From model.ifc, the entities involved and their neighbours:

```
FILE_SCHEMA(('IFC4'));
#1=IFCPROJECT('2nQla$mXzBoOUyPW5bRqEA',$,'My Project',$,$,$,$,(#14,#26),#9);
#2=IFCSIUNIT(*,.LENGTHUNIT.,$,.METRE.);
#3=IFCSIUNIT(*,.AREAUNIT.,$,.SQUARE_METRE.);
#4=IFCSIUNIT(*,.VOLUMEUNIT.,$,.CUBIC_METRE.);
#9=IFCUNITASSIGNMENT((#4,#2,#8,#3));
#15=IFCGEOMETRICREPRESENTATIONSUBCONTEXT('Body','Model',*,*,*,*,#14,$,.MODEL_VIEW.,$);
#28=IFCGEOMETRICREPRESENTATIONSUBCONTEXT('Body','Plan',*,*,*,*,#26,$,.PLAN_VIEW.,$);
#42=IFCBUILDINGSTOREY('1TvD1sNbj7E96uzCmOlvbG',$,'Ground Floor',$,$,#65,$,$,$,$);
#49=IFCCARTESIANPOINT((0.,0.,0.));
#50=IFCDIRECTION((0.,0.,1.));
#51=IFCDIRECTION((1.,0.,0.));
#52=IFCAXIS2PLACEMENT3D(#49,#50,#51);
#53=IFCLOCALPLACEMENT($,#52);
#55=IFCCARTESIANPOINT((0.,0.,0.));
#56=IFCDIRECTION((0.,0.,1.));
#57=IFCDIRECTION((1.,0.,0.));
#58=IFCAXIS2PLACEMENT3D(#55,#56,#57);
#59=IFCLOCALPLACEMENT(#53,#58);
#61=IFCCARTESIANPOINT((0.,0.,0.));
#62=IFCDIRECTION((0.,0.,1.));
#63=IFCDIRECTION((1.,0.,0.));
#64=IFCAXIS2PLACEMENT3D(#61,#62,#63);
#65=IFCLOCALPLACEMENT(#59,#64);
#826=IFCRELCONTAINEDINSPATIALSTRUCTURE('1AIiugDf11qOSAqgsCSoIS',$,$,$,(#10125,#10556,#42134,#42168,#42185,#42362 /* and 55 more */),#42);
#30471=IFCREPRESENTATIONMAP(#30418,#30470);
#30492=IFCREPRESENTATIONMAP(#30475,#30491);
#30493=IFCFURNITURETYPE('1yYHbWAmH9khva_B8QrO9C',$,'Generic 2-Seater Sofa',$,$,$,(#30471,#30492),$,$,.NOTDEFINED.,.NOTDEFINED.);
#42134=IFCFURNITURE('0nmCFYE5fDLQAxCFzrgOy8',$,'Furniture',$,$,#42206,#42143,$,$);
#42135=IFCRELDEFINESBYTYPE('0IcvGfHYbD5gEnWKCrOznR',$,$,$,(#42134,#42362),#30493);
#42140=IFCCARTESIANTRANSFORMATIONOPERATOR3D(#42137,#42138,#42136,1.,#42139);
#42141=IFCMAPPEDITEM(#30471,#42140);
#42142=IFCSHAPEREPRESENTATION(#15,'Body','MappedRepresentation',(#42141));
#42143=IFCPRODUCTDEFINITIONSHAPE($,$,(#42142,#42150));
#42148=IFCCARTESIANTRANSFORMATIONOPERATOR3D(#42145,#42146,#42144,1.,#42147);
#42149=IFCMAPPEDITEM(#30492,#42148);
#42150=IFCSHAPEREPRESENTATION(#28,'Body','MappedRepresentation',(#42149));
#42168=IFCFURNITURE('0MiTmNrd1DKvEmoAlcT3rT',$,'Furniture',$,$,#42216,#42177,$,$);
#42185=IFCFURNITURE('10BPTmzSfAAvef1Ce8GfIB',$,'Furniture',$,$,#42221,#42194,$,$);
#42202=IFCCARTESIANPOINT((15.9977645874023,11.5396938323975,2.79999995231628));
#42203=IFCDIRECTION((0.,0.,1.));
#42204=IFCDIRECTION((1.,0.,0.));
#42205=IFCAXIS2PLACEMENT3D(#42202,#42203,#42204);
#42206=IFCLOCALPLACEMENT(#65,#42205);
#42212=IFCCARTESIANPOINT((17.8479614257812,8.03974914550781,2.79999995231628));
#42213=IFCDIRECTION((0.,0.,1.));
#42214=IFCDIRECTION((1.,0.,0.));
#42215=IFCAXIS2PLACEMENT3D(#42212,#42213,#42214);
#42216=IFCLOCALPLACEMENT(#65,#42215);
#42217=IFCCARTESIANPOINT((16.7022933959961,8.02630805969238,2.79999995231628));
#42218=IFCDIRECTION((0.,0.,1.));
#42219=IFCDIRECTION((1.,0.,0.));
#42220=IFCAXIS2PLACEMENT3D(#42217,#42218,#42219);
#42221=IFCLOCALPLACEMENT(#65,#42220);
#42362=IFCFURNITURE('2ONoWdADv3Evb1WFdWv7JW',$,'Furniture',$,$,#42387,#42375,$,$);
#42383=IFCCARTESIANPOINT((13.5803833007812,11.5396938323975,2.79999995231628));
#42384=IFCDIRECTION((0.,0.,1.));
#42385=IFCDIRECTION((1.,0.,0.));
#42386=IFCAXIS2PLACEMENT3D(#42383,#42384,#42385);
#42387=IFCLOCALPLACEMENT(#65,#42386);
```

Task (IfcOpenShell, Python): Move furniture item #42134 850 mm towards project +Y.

```python
import ifcopenshell
import ifcopenshell.api.geometry
import ifcopenshell.util.placement

model = ifcopenshell.open("model.ifc")

item = model.by_id(42134)
matrix = ifcopenshell.util.placement.get_local_placement(item.ObjectPlacement)
matrix[1, 3] += 0.85
ifcopenshell.api.geometry.edit_object_placement(model, product=item, matrix=matrix, is_si=False)

print(ifcopenshell.util.placement.get_local_placement(item.ObjectPlacement).round(3) + 0.0)

model.write("model_edited.ifc")
```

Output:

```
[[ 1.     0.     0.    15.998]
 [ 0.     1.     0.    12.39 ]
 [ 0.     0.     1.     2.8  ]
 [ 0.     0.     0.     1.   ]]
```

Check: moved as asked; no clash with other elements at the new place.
